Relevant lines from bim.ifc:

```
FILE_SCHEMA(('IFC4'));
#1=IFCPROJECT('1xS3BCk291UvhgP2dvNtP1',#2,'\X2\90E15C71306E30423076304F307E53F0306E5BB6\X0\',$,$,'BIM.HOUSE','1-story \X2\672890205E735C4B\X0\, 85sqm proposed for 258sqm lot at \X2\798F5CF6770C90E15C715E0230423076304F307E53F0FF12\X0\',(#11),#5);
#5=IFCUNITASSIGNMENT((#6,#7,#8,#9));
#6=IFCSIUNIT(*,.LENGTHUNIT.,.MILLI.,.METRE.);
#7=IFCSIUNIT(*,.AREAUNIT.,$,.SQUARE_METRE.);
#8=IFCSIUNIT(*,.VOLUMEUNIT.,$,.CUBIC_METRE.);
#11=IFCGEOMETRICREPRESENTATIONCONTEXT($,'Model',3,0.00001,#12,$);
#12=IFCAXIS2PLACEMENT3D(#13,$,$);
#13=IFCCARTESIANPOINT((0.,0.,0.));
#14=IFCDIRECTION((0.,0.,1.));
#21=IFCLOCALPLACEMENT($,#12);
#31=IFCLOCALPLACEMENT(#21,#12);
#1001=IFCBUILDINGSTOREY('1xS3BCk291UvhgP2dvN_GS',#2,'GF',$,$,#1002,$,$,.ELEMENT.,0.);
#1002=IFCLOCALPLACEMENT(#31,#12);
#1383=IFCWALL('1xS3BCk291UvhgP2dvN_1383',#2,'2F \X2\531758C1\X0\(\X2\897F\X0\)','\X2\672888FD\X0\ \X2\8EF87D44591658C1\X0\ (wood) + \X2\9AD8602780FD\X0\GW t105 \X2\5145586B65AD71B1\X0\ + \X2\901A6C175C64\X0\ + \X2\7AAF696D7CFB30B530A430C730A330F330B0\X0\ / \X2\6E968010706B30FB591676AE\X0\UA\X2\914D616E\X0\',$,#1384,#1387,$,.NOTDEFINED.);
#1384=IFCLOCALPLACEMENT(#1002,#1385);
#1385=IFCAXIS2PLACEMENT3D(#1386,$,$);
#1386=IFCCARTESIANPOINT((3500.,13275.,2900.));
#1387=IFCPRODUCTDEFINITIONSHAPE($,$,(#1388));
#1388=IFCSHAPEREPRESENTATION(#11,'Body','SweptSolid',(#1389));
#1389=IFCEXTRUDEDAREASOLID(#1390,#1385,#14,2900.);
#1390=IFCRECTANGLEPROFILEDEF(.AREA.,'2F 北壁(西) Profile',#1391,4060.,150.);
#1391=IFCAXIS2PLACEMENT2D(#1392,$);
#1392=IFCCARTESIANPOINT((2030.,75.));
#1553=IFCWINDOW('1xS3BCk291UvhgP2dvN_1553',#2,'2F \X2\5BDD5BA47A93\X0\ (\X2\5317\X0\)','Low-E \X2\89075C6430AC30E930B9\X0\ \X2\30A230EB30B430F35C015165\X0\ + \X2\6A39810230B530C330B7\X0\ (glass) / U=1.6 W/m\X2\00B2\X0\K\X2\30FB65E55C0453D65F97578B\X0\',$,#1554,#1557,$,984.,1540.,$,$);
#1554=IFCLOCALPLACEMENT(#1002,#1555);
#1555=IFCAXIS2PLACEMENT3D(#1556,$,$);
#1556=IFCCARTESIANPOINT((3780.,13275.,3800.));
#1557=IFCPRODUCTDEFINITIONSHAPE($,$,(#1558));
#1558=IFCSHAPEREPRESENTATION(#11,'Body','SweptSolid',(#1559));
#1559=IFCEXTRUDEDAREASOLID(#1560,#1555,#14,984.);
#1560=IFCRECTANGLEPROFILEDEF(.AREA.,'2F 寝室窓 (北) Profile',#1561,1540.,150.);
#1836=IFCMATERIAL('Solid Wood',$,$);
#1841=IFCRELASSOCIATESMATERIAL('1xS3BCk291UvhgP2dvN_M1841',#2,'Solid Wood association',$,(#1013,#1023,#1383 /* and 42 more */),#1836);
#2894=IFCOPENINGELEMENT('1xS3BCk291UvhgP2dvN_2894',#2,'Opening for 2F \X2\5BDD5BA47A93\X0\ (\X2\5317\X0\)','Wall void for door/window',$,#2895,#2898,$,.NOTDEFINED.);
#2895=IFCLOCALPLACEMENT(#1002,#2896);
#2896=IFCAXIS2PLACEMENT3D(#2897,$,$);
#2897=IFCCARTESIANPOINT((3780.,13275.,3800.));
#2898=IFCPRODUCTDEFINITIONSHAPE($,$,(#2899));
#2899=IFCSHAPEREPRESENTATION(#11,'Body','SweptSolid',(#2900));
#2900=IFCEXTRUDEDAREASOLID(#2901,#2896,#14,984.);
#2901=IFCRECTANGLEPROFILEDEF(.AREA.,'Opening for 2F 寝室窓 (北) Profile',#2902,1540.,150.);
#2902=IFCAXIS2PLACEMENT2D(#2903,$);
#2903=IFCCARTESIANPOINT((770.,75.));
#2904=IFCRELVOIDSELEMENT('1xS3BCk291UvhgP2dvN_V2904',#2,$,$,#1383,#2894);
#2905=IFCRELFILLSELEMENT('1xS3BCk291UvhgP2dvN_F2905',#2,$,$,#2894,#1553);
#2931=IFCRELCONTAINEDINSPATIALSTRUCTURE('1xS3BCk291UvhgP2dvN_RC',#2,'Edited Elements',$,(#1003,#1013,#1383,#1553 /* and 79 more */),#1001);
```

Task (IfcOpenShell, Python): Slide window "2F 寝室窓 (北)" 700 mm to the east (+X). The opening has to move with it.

```python
import ifcopenshell
import ifcopenshell.api.geometry
import ifcopenshell.util.placement

model = ifcopenshell.open("bim.ifc")

window = model.by_guid("1xS3BCk291UvhgP2dvN_1553")
opening = window.FillsVoids[0].RelatingOpeningElement
wall = opening.VoidsElements[0].RelatingBuildingElement

wall_matrix = ifcopenshell.util.placement.get_local_placement(wall.ObjectPlacement)
shift = wall_matrix[:3, 0] * 700.0
before = ifcopenshell.util.placement.get_local_placement(window.ObjectPlacement)[:3, 3].copy()

# The window is not placed relative to its opening, so move both.
for product in (opening, window):
    matrix = ifcopenshell.util.placement.get_local_placement(product.ObjectPlacement)
    matrix[:3, 3] += shift
    ifcopenshell.api.geometry.edit_object_placement(model, product=product, matrix=matrix, is_si=False)

after = ifcopenshell.util.placement.get_local_placement(window.ObjectPlacement)[:3, 3]
print("window moved by", (after - before).round(3) + 0.0)

model.write("bim-out.ifc")
```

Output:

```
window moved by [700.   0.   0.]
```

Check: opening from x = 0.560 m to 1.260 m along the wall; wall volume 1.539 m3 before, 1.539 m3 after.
